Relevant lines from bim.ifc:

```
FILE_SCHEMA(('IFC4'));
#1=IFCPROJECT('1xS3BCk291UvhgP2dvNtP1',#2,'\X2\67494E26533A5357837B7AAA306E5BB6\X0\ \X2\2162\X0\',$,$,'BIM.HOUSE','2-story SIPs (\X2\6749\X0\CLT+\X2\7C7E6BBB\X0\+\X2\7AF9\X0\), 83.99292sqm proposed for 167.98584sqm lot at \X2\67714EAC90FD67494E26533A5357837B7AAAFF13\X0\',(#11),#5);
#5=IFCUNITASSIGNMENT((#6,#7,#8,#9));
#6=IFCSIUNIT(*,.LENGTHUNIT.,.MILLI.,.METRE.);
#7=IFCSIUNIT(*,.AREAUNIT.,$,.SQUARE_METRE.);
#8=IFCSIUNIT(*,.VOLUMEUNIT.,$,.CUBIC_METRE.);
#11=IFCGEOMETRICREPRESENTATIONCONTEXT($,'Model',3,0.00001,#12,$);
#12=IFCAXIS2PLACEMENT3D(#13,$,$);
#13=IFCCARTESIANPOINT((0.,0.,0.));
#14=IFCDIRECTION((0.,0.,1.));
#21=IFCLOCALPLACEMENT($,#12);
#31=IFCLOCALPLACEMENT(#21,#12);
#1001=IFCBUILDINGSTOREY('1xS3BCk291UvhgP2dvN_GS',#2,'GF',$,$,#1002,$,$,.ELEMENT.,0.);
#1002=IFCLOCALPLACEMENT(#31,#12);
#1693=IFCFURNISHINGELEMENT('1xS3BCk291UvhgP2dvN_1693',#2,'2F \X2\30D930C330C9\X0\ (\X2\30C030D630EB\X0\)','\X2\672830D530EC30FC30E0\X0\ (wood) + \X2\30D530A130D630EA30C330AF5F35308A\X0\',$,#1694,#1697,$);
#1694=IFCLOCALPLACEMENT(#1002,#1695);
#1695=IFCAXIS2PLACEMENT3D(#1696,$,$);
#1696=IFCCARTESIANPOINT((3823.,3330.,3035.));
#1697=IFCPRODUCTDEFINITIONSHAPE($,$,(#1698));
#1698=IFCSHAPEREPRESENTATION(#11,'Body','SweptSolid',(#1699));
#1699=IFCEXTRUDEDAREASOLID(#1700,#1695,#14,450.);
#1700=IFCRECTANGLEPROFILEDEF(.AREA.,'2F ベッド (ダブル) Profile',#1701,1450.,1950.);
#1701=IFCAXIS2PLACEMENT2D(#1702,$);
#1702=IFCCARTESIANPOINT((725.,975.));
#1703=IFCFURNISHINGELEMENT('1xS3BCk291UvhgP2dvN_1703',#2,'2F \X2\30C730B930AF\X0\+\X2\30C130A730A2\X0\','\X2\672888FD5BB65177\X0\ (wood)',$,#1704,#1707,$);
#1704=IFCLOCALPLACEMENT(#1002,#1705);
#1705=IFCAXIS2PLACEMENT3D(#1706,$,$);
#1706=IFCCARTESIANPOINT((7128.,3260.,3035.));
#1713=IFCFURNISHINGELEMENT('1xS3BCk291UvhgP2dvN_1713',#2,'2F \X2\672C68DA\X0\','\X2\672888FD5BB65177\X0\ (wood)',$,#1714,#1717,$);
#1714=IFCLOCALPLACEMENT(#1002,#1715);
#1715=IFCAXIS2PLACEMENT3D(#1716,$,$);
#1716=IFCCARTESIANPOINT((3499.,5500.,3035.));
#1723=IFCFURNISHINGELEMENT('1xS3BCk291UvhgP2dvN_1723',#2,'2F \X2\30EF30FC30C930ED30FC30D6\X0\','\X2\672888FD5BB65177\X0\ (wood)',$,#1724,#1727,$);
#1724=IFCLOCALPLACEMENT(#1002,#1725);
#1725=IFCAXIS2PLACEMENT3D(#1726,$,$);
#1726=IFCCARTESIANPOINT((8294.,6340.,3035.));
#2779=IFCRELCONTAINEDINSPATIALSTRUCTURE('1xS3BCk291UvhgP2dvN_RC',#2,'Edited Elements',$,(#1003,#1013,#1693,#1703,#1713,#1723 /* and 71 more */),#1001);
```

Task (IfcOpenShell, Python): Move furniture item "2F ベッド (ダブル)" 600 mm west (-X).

```python
import ifcopenshell
import ifcopenshell.api.geometry
import ifcopenshell.util.placement

model = ifcopenshell.open("bim.ifc")

item = model.by_guid("1xS3BCk291UvhgP2dvN_1693")
matrix = ifcopenshell.util.placement.get_local_placement(item.ObjectPlacement)
matrix[0, 3] -= 600.0
ifcopenshell.api.geometry.edit_object_placement(model, product=item, matrix=matrix, is_si=False)

print(ifcopenshell.util.placement.get_local_placement(item.ObjectPlacement).round(3) + 0.0)

model.write("bim_updated.ifc")
```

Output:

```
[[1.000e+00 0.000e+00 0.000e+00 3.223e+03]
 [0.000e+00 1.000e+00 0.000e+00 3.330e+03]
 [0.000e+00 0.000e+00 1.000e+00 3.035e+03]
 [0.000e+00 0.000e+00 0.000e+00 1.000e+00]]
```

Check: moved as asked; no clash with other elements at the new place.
